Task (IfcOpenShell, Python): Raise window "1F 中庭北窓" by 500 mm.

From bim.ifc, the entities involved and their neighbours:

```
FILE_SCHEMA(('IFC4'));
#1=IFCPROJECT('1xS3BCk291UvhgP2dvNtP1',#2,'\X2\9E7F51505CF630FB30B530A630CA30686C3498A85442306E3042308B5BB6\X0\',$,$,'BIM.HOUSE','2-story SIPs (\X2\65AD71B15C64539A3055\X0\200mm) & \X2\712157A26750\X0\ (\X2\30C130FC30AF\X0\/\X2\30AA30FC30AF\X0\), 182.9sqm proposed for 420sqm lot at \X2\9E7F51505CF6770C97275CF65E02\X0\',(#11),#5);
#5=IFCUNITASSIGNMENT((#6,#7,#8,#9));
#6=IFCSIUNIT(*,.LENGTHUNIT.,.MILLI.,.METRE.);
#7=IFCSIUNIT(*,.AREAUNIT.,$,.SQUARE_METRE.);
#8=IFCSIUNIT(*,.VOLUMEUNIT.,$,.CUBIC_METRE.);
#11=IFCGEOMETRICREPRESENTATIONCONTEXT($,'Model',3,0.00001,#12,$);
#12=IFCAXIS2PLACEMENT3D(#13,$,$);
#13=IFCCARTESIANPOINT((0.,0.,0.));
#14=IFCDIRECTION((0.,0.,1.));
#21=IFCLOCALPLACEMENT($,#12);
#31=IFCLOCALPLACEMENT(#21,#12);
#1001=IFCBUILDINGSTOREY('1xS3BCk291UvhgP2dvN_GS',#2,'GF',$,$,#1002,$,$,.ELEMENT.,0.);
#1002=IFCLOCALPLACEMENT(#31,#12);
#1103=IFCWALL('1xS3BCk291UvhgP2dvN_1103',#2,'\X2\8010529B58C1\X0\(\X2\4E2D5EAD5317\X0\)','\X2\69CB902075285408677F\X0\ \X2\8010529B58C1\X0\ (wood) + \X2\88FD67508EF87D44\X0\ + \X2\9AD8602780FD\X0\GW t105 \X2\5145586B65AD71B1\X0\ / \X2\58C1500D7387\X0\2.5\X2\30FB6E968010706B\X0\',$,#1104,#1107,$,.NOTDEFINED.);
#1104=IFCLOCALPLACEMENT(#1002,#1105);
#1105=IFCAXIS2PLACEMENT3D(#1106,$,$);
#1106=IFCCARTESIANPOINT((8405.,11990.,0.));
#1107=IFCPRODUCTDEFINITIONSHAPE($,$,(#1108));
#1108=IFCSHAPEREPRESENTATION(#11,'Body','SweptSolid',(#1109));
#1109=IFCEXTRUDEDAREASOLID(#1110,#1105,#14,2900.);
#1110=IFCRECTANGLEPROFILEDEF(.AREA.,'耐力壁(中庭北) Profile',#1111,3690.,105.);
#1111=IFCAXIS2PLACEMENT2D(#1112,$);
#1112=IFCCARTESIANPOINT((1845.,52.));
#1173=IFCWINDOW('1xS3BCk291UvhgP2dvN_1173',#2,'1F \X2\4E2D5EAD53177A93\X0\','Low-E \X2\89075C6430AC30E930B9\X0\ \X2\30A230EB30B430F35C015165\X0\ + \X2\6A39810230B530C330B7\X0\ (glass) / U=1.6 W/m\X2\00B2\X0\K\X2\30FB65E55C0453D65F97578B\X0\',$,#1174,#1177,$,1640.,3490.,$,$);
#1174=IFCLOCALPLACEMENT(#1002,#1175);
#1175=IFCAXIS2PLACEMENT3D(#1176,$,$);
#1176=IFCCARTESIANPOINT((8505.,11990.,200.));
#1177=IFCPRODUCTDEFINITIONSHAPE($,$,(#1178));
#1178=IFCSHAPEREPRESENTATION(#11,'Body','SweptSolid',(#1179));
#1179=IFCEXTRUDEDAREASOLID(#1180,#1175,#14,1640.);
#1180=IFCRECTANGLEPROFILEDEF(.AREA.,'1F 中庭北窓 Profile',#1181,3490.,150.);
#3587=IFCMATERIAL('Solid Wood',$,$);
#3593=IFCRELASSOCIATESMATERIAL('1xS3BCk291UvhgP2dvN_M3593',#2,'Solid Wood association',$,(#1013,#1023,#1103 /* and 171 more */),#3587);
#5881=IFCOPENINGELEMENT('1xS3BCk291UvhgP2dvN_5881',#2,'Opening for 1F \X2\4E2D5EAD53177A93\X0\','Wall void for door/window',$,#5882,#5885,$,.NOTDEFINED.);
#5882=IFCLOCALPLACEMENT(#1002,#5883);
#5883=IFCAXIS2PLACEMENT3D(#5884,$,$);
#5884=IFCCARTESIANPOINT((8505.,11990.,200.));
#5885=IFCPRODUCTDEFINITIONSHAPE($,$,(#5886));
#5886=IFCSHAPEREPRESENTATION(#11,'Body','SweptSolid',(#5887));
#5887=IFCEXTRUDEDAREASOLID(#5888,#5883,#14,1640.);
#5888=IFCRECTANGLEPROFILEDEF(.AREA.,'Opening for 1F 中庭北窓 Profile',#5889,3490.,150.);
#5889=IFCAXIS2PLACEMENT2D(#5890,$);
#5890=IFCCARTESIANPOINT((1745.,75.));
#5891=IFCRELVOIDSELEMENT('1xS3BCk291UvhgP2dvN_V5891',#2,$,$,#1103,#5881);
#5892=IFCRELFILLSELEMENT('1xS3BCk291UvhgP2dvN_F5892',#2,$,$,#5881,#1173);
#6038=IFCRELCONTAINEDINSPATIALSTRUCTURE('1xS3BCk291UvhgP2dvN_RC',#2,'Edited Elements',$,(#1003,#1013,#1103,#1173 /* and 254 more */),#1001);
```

```python
import numpy as np
import ifcopenshell
import ifcopenshell.api.geometry
import ifcopenshell.util.placement
import ifcopenshell.util.unit

model = ifcopenshell.open("bim.ifc")
unit_scale = ifcopenshell.util.unit.calculate_unit_scale(model)

window = model.by_guid("1xS3BCk291UvhgP2dvN_1173")
opening = window.FillsVoids[0].RelatingOpeningElement
dz = 500.0

shift = np.array([0.0, 0.0, dz])
# The window is not placed relative to its opening, so move both.
for product in (opening, window):
    matrix = ifcopenshell.util.placement.get_local_placement(product.ObjectPlacement)
    matrix[:3, 3] += shift
    ifcopenshell.api.geometry.edit_object_placement(model, product=product, matrix=matrix, is_si=False)

print(f"moved by {dz * unit_scale:+.3f} m")

model.write("bim_updated.ifc")
```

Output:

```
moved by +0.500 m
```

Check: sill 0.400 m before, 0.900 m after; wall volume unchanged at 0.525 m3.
